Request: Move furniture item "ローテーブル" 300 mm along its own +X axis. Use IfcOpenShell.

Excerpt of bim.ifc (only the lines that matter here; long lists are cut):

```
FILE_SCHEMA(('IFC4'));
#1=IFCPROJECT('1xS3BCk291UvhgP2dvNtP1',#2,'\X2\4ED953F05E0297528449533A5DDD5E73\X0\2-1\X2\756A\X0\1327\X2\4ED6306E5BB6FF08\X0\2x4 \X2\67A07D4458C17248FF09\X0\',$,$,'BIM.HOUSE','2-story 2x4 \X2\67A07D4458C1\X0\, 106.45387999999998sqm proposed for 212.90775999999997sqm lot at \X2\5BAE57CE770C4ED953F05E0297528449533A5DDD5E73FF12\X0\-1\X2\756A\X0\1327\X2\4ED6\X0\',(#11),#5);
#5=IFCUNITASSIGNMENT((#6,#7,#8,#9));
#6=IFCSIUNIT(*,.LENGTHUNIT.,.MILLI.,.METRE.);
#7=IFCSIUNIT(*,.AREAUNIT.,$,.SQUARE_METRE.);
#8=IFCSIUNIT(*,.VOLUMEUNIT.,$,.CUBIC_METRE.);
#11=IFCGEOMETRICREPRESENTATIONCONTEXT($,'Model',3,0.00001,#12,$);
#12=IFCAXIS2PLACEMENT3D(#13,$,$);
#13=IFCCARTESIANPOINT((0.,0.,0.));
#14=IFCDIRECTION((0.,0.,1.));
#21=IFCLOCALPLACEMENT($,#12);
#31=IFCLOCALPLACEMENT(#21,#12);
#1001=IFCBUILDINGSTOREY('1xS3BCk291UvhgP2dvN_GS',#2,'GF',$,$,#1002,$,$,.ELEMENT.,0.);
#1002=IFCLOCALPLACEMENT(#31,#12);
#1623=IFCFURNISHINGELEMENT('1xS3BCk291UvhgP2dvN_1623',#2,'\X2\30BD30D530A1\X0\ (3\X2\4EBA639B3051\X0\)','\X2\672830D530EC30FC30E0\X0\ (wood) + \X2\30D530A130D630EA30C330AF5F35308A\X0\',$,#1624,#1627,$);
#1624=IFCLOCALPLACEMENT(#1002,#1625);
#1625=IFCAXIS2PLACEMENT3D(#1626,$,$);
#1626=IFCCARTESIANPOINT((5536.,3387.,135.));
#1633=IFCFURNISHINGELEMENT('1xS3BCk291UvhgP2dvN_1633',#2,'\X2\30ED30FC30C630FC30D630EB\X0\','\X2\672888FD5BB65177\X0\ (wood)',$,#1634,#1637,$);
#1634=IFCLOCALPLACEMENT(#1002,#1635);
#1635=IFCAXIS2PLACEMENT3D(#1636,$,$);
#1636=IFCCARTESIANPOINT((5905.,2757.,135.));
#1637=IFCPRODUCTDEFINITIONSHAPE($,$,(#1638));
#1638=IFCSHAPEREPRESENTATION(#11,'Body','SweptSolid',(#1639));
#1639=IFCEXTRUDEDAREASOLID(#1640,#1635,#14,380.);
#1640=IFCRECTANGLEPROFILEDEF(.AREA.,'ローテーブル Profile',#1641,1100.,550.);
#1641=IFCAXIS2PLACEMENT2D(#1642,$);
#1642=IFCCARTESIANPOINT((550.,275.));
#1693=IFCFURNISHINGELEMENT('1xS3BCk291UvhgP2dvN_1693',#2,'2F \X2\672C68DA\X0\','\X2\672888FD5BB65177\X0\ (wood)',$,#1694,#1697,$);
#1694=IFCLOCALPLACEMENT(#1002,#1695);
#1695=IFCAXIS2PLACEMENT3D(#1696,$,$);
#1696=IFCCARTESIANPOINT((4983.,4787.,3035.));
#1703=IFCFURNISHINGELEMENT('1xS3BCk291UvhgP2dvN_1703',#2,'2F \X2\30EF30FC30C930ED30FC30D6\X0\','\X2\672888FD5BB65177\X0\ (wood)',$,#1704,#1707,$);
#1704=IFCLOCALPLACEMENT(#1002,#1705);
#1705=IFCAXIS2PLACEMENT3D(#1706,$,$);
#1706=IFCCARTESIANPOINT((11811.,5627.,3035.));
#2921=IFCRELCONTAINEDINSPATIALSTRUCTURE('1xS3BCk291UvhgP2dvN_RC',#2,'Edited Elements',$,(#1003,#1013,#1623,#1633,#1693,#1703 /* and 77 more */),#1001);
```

```python
import ifcopenshell
import ifcopenshell.api.geometry
import ifcopenshell.util.placement

model = ifcopenshell.open("bim.ifc")

item = model.by_guid("1xS3BCk291UvhgP2dvN_1633")
matrix = ifcopenshell.util.placement.get_local_placement(item.ObjectPlacement)
matrix[:3, 3] += matrix[:3, 0] * 300.0
ifcopenshell.api.geometry.edit_object_placement(model, product=item, matrix=matrix, is_si=False)

print(ifcopenshell.util.placement.get_local_placement(item.ObjectPlacement).round(3) + 0.0)

model.write("bim_edited.ifc")
```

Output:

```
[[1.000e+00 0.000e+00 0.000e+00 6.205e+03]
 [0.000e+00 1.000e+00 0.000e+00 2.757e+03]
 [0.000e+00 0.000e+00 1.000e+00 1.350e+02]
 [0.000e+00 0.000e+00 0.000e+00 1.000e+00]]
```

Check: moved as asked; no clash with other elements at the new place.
